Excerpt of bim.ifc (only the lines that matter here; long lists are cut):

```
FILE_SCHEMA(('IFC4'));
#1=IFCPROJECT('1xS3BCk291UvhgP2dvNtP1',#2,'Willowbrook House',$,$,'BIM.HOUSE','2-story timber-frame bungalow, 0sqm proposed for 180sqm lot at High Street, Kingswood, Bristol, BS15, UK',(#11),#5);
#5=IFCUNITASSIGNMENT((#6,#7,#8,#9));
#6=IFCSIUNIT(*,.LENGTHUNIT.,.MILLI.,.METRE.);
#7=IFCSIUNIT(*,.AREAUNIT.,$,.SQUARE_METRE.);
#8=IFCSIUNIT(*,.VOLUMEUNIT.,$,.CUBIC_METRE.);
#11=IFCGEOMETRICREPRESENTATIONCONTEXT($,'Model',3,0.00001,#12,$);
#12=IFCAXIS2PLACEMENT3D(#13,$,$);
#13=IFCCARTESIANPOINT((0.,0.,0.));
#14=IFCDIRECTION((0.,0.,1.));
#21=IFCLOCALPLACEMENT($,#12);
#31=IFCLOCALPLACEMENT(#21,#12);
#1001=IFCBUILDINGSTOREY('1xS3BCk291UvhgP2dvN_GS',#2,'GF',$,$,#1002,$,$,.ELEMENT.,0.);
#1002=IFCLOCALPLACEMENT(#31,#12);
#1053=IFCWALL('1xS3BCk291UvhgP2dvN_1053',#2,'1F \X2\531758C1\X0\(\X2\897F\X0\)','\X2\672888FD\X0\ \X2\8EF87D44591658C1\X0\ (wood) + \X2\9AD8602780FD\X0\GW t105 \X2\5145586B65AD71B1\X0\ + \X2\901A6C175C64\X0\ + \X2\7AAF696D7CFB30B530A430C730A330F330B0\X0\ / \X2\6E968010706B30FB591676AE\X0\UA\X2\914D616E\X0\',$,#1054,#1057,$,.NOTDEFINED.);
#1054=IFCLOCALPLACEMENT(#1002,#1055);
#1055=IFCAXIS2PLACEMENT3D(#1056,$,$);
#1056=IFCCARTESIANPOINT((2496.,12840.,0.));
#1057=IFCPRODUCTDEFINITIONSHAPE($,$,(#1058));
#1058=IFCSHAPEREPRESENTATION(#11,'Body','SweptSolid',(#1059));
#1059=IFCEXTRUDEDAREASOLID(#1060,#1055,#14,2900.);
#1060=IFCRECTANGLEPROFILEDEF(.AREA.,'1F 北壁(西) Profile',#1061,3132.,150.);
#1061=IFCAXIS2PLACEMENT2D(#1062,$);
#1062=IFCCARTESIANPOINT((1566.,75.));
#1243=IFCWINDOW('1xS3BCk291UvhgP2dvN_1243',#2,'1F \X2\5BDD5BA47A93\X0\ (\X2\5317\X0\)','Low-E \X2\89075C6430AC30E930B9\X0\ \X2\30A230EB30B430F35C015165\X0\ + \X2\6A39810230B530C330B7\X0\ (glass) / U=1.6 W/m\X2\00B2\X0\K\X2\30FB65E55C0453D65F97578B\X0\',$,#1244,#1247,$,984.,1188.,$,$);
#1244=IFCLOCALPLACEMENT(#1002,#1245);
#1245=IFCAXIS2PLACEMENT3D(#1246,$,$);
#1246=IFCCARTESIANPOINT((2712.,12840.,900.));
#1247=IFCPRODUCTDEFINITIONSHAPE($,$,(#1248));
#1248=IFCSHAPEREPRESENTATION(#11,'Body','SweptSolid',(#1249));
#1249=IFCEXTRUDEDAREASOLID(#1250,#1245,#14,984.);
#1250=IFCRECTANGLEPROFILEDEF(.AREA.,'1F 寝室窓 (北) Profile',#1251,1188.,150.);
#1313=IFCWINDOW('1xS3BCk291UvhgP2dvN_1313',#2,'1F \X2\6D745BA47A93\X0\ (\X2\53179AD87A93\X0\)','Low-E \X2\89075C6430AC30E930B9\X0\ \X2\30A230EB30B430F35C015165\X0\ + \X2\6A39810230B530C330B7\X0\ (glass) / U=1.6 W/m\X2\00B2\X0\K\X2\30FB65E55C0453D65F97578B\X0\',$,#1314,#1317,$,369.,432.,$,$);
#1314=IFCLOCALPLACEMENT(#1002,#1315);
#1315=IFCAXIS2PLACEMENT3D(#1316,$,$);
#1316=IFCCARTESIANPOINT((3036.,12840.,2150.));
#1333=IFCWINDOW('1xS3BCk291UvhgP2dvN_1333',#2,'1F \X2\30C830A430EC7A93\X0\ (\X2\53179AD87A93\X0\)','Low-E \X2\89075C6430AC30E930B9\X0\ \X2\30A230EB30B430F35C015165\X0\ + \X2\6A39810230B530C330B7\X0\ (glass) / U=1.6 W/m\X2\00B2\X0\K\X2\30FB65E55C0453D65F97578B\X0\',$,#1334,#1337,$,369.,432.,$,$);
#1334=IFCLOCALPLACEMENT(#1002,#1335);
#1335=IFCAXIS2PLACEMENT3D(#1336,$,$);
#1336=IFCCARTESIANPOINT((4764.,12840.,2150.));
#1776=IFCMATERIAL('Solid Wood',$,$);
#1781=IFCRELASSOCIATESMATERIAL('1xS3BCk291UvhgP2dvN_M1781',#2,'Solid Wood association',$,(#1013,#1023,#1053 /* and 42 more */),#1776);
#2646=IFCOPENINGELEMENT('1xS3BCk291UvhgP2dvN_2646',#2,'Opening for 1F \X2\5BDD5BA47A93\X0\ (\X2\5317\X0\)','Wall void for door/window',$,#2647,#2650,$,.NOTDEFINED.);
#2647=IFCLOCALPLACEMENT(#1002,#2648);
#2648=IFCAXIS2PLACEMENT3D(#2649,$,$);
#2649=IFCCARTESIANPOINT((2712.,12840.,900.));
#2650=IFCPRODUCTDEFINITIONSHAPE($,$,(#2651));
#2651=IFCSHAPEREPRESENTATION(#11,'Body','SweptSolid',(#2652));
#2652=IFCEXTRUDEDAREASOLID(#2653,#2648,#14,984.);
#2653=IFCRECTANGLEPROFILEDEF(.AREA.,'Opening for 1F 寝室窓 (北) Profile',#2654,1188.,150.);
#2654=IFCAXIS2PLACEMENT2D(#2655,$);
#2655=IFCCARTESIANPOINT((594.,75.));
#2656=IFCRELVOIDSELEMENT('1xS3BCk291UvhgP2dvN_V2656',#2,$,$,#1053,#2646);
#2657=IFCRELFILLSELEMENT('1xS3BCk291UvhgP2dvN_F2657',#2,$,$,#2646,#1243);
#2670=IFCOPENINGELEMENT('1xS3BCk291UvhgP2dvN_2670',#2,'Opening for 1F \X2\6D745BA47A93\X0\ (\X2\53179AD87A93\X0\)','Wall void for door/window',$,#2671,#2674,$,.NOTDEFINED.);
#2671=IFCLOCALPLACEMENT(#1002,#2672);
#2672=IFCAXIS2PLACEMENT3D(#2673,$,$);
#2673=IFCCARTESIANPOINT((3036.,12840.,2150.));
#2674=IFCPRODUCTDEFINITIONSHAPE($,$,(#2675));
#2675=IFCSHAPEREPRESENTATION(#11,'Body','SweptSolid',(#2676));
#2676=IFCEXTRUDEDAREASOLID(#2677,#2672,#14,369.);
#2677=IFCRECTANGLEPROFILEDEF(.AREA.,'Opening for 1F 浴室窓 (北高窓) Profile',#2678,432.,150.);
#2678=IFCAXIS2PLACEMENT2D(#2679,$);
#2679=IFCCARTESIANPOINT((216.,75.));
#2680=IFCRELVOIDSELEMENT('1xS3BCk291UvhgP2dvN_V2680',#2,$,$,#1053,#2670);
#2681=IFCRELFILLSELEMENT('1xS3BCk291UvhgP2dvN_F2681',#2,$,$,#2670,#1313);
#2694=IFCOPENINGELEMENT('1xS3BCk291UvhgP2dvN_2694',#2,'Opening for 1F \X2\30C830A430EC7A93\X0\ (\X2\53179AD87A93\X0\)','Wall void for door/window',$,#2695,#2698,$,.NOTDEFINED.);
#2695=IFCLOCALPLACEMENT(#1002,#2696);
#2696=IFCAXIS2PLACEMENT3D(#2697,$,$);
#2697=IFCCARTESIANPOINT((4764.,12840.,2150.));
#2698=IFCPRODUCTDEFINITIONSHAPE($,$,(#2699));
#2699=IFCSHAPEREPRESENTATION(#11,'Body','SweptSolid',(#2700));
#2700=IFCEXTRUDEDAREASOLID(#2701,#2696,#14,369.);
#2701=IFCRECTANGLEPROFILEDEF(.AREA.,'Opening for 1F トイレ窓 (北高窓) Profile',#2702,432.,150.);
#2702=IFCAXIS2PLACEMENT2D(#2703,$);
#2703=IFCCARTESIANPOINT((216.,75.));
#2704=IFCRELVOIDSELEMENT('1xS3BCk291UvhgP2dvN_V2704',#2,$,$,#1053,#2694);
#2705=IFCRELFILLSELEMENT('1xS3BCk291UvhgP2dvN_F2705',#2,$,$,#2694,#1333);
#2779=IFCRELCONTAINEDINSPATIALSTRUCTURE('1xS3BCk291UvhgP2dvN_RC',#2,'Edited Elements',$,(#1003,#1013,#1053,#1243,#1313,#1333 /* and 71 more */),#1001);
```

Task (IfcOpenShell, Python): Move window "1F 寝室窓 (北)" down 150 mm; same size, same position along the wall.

```python
import numpy as np
import ifcopenshell
import ifcopenshell.api.geometry
import ifcopenshell.util.placement
import ifcopenshell.util.unit

model = ifcopenshell.open("bim.ifc")
unit_scale = ifcopenshell.util.unit.calculate_unit_scale(model)

window = model.by_id(1243)
opening = window.FillsVoids[0].RelatingOpeningElement
dz = -0.15 / unit_scale

shift = np.array([0.0, 0.0, dz])
# The window is not placed relative to its opening, so move both.
for product in (opening, window):
    matrix = ifcopenshell.util.placement.get_local_placement(product.ObjectPlacement)
    matrix[:3, 3] += shift
    ifcopenshell.api.geometry.edit_object_placement(model, product=product, matrix=matrix, is_si=False)

print(f"moved by {dz * unit_scale:+.3f} m")

model.write("bim_edited.ifc")
```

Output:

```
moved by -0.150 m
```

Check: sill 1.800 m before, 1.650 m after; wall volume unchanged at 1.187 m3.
